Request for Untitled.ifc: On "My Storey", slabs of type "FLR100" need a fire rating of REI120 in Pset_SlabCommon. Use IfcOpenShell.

First a look at what the model holds.

```python
import ifcopenshell
import ifcopenshell.util.element

model = ifcopenshell.open("Untitled.ifc")
print(model.schema)
storey = next(s for s in model.by_type("IfcBuildingStorey") if s.Name == "My Storey")
slabs = [e for e in ifcopenshell.util.element.get_decomposition(storey) if e.is_a("IfcSlab")]
seen = {}
for e in slabs:
    element_type = ifcopenshell.util.element.get_type(e)
    key = (element_type.Name if element_type != e and element_type else None, ifcopenshell.util.element.get_pset(e, "Pset_SlabCommon", "FireRating"))
    seen[key] = seen.get(key, 0) + 1
for (name, value), count in sorted(seen.items(), key=str):
    print(count, "x", name, "|", value)
```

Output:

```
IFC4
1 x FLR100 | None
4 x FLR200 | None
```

```python
import ifcopenshell
import ifcopenshell.api.pset
import ifcopenshell.util.element

model = ifcopenshell.open("Untitled.ifc")

storey = next(s for s in model.by_type("IfcBuildingStorey") if s.Name == "My Storey")
slabs = [e for e in ifcopenshell.util.element.get_decomposition(storey) if e.is_a("IfcSlab")]

count = 0
for e in slabs:
    element_type = ifcopenshell.util.element.get_type(e)
    if element_type in (None, e) or element_type.Name != "FLR100":
        continue
    # add_pset returns the element's existing set when there is one.
    pset = ifcopenshell.api.pset.add_pset(model, product=e, name="Pset_SlabCommon")
    ifcopenshell.api.pset.edit_pset(model, pset=pset, properties={"FireRating": "REI120"})
    count += 1

print(count, "slabs updated")

model.write("Untitled_updated.ifc")
```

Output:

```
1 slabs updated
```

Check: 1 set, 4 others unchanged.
